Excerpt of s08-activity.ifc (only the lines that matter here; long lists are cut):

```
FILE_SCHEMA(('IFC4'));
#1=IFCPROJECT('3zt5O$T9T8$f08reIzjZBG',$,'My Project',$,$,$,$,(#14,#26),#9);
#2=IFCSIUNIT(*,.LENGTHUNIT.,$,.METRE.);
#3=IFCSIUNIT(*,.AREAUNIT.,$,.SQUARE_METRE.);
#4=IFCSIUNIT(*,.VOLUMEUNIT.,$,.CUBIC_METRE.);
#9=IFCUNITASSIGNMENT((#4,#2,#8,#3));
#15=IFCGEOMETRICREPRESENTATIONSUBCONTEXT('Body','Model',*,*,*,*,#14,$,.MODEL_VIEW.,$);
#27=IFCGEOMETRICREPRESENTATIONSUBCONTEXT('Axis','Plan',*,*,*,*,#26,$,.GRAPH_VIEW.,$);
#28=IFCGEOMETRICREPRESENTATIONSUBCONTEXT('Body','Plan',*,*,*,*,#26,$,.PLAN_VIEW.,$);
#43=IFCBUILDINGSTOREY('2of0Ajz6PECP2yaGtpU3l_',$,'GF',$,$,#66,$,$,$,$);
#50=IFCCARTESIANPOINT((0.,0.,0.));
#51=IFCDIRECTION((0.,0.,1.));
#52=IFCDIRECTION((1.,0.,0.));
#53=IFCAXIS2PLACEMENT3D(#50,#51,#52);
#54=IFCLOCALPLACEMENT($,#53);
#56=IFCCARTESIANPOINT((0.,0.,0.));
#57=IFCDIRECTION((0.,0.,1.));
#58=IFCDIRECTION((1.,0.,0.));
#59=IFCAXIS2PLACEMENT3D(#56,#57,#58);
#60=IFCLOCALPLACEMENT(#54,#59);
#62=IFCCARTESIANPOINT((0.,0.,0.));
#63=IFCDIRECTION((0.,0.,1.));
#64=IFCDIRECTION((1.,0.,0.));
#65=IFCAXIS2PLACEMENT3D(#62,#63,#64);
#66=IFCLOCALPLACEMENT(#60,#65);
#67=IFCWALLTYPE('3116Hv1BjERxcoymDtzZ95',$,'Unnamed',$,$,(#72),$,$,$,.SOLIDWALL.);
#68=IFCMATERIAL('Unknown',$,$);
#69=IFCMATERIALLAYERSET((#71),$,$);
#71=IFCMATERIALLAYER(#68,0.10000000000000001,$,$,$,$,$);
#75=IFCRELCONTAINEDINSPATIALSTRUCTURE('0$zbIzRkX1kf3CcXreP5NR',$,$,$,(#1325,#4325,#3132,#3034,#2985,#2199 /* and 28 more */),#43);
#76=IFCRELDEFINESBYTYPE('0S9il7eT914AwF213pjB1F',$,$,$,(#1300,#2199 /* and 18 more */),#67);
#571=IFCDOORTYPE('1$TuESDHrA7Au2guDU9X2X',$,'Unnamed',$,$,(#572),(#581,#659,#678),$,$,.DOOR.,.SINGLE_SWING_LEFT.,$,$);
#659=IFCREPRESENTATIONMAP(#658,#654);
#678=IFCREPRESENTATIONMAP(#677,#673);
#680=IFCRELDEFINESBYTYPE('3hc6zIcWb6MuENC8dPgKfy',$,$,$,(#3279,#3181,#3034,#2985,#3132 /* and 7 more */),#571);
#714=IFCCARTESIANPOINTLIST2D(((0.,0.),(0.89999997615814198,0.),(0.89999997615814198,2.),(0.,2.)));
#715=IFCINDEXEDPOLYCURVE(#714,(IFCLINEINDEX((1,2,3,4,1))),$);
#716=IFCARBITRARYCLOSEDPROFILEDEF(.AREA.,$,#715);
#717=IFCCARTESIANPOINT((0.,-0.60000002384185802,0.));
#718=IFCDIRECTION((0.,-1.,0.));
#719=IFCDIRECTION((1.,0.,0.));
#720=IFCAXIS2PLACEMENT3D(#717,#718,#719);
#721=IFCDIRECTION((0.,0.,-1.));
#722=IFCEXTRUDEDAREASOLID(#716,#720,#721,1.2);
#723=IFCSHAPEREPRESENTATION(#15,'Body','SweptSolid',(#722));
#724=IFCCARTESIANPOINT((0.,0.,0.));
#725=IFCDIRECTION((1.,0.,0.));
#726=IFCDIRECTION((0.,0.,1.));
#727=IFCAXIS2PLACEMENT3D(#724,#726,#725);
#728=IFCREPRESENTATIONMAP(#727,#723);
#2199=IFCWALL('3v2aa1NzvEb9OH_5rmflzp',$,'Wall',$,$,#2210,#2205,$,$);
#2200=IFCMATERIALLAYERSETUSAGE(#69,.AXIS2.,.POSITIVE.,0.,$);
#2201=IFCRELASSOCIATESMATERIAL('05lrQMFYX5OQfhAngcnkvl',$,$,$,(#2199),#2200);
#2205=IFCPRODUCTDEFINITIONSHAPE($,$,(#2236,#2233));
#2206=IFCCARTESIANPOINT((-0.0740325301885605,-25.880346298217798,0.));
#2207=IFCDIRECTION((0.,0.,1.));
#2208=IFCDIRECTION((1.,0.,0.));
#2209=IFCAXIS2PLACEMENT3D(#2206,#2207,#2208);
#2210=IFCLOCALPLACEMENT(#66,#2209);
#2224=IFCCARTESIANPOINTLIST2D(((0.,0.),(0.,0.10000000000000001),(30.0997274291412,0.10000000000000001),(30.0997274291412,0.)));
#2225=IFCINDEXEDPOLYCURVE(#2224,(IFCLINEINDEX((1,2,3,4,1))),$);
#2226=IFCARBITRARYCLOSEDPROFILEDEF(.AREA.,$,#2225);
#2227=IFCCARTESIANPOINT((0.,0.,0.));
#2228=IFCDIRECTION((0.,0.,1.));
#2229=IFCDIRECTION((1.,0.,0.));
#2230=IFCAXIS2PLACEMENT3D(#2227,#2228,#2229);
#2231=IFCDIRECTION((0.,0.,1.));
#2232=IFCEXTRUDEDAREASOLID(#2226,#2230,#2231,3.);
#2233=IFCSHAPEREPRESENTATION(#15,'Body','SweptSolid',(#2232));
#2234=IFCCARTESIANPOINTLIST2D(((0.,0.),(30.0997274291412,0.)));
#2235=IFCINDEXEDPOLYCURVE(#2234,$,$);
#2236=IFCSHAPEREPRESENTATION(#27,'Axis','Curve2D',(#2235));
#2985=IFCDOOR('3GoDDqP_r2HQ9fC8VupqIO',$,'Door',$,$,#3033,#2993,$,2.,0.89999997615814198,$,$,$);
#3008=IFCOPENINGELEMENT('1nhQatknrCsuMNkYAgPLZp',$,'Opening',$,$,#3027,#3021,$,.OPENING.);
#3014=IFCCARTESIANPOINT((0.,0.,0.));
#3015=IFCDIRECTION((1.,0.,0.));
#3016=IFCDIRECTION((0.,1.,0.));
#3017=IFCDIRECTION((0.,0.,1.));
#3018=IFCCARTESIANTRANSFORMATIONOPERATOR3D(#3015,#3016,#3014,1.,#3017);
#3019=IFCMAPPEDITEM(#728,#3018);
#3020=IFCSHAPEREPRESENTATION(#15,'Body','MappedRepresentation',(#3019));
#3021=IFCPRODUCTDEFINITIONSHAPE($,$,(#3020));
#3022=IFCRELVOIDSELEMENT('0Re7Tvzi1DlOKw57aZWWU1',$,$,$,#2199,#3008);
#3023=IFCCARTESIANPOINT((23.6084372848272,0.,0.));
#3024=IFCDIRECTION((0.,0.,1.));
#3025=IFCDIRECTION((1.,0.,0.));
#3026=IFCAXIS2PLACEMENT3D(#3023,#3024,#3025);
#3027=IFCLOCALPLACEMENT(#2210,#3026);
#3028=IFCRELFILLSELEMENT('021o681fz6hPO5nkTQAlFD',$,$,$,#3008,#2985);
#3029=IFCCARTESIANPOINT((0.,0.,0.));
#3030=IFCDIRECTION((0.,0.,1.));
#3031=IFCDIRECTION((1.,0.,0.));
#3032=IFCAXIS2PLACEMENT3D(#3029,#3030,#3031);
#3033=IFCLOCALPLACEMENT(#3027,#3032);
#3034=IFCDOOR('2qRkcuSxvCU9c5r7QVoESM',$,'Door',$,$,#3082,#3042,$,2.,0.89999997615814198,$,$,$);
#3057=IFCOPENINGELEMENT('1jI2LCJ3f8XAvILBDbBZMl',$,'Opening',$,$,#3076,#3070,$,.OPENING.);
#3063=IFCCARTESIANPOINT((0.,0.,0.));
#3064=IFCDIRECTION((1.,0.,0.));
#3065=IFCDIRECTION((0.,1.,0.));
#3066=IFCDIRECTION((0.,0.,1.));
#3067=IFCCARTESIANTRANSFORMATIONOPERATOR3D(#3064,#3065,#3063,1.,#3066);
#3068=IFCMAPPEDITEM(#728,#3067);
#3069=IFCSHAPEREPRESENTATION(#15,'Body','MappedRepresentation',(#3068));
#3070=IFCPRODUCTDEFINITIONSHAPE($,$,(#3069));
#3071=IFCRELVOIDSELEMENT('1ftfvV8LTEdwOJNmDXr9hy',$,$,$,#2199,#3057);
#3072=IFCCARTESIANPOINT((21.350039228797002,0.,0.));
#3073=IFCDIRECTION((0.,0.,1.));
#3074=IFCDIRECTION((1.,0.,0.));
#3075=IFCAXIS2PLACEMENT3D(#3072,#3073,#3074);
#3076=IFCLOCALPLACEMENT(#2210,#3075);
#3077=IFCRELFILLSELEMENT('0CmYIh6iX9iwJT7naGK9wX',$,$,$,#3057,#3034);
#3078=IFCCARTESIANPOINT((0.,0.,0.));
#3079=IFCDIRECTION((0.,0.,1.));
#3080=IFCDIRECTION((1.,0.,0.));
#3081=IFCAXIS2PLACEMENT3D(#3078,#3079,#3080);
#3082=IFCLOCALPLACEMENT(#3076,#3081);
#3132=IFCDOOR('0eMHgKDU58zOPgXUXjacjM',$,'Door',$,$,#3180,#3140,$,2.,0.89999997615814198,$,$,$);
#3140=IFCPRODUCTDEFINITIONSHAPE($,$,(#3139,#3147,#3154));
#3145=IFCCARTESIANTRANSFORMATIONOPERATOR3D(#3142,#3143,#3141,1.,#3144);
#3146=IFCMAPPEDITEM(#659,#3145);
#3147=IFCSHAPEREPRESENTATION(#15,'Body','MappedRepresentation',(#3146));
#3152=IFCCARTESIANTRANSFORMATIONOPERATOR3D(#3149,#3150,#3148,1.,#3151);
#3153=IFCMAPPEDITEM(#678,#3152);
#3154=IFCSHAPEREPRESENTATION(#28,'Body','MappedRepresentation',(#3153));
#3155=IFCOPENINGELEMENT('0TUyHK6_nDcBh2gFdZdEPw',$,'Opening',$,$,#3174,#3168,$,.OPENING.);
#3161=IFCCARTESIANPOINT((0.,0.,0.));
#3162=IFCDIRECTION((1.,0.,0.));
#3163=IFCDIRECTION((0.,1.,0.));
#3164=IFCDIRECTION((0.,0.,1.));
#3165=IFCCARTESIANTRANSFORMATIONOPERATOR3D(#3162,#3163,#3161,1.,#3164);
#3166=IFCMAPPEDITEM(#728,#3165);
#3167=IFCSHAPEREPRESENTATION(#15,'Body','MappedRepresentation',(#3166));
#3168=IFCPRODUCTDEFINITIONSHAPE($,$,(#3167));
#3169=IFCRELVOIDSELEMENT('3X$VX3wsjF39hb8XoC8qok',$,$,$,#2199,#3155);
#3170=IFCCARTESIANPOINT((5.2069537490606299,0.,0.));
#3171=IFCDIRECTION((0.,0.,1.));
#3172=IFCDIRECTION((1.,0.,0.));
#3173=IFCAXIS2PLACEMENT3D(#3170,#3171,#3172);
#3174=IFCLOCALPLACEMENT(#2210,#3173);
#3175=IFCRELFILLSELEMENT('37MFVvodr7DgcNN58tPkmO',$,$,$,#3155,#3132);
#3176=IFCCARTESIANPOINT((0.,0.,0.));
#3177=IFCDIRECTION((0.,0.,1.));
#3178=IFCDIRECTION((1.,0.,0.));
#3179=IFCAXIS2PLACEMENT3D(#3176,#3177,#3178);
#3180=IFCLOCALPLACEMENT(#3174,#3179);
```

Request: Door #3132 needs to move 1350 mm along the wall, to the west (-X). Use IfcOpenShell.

```python
import ifcopenshell
import ifcopenshell.api.geometry
import ifcopenshell.util.placement
import ifcopenshell.util.unit

model = ifcopenshell.open("s08-activity.ifc")
unit_scale = ifcopenshell.util.unit.calculate_unit_scale(model)

door = model.by_guid("0eMHgKDU58zOPgXUXjacjM")
opening = door.FillsVoids[0].RelatingOpeningElement
wall = opening.VoidsElements[0].RelatingBuildingElement

wall_matrix = ifcopenshell.util.placement.get_local_placement(wall.ObjectPlacement)
shift = wall_matrix[:3, 0] * -1.35 / unit_scale
before = ifcopenshell.util.placement.get_local_placement(door.ObjectPlacement)[:3, 3].copy()

# The door is placed relative to its opening, so it follows when the opening moves.
matrix = ifcopenshell.util.placement.get_local_placement(opening.ObjectPlacement)
matrix[:3, 3] += shift
ifcopenshell.api.geometry.edit_object_placement(
    model, product=opening, matrix=matrix, is_si=False, should_transform_children=True
)

after = ifcopenshell.util.placement.get_local_placement(door.ObjectPlacement)[:3, 3]
print("door moved by", (after - before).round(3) + 0.0)

model.write("s08-activity_edited.ifc")
```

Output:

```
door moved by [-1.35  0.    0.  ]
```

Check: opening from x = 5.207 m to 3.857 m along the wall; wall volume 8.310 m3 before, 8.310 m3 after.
